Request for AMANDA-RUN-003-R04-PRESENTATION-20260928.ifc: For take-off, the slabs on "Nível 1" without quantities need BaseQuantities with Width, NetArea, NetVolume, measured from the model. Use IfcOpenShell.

First a look at what the model holds.

```python
import ifcopenshell
import ifcopenshell.util.element
import ifcopenshell.util.unit

model = ifcopenshell.open("AMANDA-RUN-003-R04-PRESENTATION-20260928.ifc")
print(model.schema)
for unit_type in ("LENGTHUNIT", "AREAUNIT", "VOLUMEUNIT"):
    print(unit_type, ifcopenshell.util.unit.calculate_unit_scale(model, unit_type))
storey = next(s for s in model.by_type("IfcBuildingStorey") if s.Name == "Nível 1")
slabs = [e for e in ifcopenshell.util.element.get_decomposition(storey) if e.is_a("IfcSlab")]
for e in sorted(slabs, key=lambda e: e.id()):
    print(e.id(), e.is_a(), e.Name, list(ifcopenshell.util.element.get_psets(e, qtos_only=True)), sep=" | ")
```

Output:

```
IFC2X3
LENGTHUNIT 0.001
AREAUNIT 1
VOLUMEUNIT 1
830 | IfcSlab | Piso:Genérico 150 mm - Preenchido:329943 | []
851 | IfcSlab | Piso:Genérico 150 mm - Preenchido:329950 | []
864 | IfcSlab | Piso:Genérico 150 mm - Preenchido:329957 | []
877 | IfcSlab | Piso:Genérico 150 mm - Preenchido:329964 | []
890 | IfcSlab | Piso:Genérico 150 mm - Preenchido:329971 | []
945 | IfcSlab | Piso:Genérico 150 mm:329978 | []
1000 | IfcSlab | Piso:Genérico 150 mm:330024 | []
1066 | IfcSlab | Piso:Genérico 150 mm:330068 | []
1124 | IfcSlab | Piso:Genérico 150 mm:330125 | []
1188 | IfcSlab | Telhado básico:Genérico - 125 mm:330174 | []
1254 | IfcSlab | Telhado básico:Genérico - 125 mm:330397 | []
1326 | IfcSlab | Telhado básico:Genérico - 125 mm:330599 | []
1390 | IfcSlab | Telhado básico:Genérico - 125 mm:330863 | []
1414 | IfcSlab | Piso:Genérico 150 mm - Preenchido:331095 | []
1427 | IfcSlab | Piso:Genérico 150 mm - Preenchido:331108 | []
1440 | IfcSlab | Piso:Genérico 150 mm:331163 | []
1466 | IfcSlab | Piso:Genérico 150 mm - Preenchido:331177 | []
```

```python
import ifcopenshell
import ifcopenshell.api.pset
import ifcopenshell.geom
import ifcopenshell.util.element
import ifcopenshell.util.shape
import ifcopenshell.util.unit

model = ifcopenshell.open("AMANDA-RUN-003-R04-PRESENTATION-20260928.ifc")
unit_scale = ifcopenshell.util.unit.calculate_unit_scale(model)
area_scale = ifcopenshell.util.unit.calculate_unit_scale(model, "AREAUNIT")
volume_scale = ifcopenshell.util.unit.calculate_unit_scale(model, "VOLUMEUNIT")
settings = ifcopenshell.geom.settings()

storey = next(s for s in model.by_type("IfcBuildingStorey") if s.Name == "Nível 1")
slabs = [e for e in ifcopenshell.util.element.get_decomposition(storey) if e.is_a("IfcSlab")]

for e in sorted(slabs, key=lambda e: e.id()):
    if ifcopenshell.util.element.get_psets(e, qtos_only=True, should_inherit=False):
        continue
    # Geometry comes back in metres, in the element's own axes.
    shape = ifcopenshell.geom.create_shape(settings, e)
    values = {
        "Width": ifcopenshell.util.shape.get_z(shape.geometry) / unit_scale,
        "NetArea": ifcopenshell.util.shape.get_footprint_area(shape.geometry) / area_scale,
        "NetVolume": ifcopenshell.util.shape.get_volume(shape.geometry) / volume_scale,
    }
    qto = ifcopenshell.api.pset.add_qto(model, product=e, name="BaseQuantities")
    ifcopenshell.api.pset.edit_qto(model, qto=qto, properties=values)
    print(e.id(), {k: round(v, 3) for k, v in values.items()})

model.write("AMANDA-RUN-003-R04-PRESENTATION-20260928_rev.ifc")
```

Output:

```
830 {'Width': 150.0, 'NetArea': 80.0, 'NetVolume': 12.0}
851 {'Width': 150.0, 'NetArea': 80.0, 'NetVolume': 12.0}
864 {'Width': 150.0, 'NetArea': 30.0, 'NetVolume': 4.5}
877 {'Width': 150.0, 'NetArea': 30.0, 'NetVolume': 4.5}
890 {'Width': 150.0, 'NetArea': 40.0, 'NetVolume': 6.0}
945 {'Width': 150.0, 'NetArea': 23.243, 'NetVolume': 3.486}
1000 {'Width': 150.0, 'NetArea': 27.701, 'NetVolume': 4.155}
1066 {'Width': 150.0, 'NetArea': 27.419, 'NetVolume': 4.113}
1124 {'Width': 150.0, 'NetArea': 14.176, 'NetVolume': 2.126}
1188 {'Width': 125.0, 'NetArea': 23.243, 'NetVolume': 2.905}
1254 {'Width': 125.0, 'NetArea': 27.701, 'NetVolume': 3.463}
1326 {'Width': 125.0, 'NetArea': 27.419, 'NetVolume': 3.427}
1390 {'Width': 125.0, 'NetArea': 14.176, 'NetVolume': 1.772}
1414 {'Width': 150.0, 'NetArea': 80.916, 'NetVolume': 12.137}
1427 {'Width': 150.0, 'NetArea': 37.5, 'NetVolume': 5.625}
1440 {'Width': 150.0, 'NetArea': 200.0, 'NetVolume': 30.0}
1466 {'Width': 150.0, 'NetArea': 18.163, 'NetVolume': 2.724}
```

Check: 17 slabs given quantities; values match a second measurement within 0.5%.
